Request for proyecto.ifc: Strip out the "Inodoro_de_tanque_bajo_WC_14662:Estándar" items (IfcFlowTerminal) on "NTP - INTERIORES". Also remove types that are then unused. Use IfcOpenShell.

First a look at what the model holds.

```python
import ifcopenshell
import ifcopenshell.util.element

model = ifcopenshell.open("proyecto.ifc")
print(model.schema)
storey = next(s for s in model.by_type("IfcBuildingStorey") if s.Name == "NTP - INTERIORES")
terminals = [e for e in ifcopenshell.util.element.get_decomposition(storey) if e.is_a("IfcFlowTerminal")]
seen = {}
for e in terminals:
    element_type = ifcopenshell.util.element.get_type(e)
    name = element_type.Name if element_type not in (None, e) else None
    seen[name] = seen.get(name, 0) + 1
for name, count in sorted(seen.items(), key=str):
    print(count, "x", name)
```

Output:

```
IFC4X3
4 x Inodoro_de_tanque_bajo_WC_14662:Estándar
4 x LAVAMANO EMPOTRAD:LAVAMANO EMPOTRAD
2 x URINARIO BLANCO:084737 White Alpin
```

```python
import ifcopenshell
import ifcopenshell.api.root
import ifcopenshell.util.element

model = ifcopenshell.open("proyecto.ifc")

storey = next(s for s in model.by_type("IfcBuildingStorey") if s.Name == "NTP - INTERIORES")
terminals = [e for e in ifcopenshell.util.element.get_decomposition(storey) if e.is_a("IfcFlowTerminal")]
targets = [e for e in terminals if (t := ifcopenshell.util.element.get_type(e)) not in (None, e) and t.Name == "Inodoro_de_tanque_bajo_WC_14662:Estándar"]
types = {ifcopenshell.util.element.get_type(e) for e in targets} - {None, *targets}

for e in targets:
    ifcopenshell.api.root.remove_product(model, product=e)
print(len(targets), "removed")

unused = [t for t in types if not ifcopenshell.util.element.get_types(t)]
for t in unused:
    ifcopenshell.api.root.remove_product(model, product=t)
print(len(unused), "unused types removed")

model.write("proyecto_rev.ifc")
```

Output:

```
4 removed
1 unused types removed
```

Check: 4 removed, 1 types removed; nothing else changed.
